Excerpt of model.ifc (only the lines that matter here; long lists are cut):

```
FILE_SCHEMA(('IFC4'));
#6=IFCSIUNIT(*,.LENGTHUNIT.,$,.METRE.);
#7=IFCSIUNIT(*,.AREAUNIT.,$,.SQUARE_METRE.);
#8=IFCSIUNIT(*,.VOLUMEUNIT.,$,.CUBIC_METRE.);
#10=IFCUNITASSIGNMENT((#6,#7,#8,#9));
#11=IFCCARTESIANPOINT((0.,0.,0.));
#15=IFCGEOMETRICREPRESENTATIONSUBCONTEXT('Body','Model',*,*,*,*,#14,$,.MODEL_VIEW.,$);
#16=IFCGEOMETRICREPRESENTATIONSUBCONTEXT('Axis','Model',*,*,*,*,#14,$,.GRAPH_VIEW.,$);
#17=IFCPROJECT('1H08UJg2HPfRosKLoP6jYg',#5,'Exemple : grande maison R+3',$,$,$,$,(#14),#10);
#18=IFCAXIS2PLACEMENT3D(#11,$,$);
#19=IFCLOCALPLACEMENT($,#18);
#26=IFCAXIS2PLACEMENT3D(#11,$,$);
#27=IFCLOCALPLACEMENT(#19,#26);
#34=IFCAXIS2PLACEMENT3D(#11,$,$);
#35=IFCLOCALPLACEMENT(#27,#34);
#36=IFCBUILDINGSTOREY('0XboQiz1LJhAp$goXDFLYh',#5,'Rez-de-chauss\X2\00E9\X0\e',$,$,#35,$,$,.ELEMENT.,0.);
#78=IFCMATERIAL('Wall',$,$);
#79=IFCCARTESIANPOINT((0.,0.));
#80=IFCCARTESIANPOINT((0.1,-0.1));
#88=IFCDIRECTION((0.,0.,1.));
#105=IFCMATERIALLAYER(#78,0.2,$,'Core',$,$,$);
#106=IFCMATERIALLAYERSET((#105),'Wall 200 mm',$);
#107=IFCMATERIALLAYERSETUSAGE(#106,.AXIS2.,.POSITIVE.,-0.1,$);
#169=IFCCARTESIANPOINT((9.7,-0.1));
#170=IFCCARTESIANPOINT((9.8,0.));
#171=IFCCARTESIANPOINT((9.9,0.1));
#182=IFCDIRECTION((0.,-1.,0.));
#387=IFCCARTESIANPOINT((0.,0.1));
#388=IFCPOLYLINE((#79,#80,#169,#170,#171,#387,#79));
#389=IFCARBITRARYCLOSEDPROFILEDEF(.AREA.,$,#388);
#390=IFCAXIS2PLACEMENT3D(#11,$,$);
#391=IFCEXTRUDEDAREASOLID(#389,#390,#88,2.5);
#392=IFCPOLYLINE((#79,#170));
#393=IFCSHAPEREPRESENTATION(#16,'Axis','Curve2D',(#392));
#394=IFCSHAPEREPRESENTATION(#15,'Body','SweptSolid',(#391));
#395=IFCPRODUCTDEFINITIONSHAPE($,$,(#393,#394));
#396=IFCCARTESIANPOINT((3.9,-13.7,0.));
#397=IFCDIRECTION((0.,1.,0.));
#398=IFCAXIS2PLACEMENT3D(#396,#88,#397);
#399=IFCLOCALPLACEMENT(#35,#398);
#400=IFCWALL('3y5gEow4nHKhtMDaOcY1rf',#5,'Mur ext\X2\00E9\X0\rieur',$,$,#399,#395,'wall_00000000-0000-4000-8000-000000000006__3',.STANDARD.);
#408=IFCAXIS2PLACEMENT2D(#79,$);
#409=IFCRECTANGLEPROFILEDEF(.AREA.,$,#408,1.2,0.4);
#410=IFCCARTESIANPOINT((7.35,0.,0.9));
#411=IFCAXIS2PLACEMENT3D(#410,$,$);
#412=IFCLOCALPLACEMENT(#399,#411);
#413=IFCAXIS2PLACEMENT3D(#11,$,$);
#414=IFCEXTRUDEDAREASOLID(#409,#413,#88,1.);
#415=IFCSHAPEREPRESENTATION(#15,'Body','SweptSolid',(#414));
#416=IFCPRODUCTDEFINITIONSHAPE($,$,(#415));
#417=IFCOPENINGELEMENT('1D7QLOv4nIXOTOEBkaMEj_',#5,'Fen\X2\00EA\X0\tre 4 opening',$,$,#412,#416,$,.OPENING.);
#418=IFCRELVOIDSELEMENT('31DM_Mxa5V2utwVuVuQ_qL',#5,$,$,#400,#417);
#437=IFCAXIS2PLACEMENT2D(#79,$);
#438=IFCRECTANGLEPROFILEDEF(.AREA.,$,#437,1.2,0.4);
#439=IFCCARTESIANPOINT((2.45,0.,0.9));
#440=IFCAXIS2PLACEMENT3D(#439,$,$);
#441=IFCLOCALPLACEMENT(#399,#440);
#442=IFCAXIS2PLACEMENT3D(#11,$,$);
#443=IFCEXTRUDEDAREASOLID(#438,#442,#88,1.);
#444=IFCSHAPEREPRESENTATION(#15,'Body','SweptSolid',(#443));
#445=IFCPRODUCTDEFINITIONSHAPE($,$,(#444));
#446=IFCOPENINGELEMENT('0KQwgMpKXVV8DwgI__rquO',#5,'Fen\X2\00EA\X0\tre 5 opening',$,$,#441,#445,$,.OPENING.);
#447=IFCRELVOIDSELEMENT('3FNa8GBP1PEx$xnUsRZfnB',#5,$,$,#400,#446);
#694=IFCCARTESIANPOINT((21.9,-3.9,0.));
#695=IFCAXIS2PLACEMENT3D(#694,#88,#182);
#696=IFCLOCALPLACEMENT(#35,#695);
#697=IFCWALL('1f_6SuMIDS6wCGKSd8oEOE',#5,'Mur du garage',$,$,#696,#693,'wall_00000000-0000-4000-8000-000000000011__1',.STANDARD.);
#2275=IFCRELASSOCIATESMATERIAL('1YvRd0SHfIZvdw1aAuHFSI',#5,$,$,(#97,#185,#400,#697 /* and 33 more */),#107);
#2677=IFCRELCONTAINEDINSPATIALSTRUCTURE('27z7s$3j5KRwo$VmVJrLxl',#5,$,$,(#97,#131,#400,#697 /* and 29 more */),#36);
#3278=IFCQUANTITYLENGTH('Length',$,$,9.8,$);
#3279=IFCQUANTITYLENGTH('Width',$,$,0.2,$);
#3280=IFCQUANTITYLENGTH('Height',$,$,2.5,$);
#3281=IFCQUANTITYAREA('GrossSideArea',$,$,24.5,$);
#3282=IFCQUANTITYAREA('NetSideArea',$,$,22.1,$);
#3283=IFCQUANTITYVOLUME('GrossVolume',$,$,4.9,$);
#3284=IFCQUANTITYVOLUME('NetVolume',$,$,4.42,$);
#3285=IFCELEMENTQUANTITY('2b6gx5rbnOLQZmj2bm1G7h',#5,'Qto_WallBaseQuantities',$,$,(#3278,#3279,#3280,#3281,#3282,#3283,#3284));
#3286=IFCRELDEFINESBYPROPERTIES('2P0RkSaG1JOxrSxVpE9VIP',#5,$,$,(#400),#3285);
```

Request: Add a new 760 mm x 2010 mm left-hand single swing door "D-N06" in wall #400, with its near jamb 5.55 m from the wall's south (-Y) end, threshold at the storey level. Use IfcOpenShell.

```python
import numpy as np
import ifcopenshell
import ifcopenshell.api.feature
import ifcopenshell.api.geometry
import ifcopenshell.api.pset
import ifcopenshell.api.root
import ifcopenshell.api.spatial
import ifcopenshell.geom
import ifcopenshell.util.element
import ifcopenshell.util.placement
import ifcopenshell.util.representation
import ifcopenshell.util.shape
import ifcopenshell.util.unit

model = ifcopenshell.open("model.ifc")
unit_scale = ifcopenshell.util.unit.calculate_unit_scale(model)
area_scale = ifcopenshell.util.unit.calculate_unit_scale(model, "AREAUNIT")
volume_scale = ifcopenshell.util.unit.calculate_unit_scale(model, "VOLUMEUNIT")
settings = ifcopenshell.geom.settings()


def volume(element):
    """Net volume in cubic metres, openings subtracted."""
    shape = ifcopenshell.geom.create_shape(settings, element)
    return ifcopenshell.util.shape.get_volume(shape.geometry)


wall = model.by_id(400)
storey = ifcopenshell.util.element.get_container(wall, ifc_class="IfcBuildingStorey")
context = ifcopenshell.util.representation.get_context(model, "Model", "Body", "MODEL_VIEW")
before = volume(wall)

width, height, from_end, sill = 0.76, 2.01, 5.55, 0.0  # metres

# The wall runs along its own X axis, and the end named is its -X end.
wall_shape = ifcopenshell.geom.create_shape(settings, wall)
x, y, z = ifcopenshell.util.shape.get_vertices(wall_shape.geometry).T
start = x.min() + from_end
face, thickness = float(y.min()), float(y.max() - y.min())
wall_matrix = ifcopenshell.util.placement.get_local_placement(wall.ObjectPlacement)
level = ifcopenshell.util.placement.get_local_placement(storey.ObjectPlacement)[2, 3]


def in_wall(x, y):
    """Placement at x, y metres in the wall's axes, at sill height."""
    matrix = wall_matrix.copy()
    matrix[:, 3] = wall_matrix @ np.array([x / unit_scale, y / unit_scale, 0.0, 1.0])
    matrix[2, 3] = level + sill / unit_scale
    return matrix


# Opening: a box that overshoots both wall faces by 50 mm.
opening = ifcopenshell.api.root.create_entity(model, ifc_class="IfcOpeningElement", predefined_type="OPENING")
box = ifcopenshell.api.geometry.add_wall_representation(
    model, context=context, length=width, height=height, thickness=thickness + 0.1
)
ifcopenshell.api.geometry.assign_representation(model, product=opening, representation=box)
ifcopenshell.api.geometry.edit_object_placement(model, product=opening, matrix=in_wall(start, face - 0.05), is_si=False)
ifcopenshell.api.feature.add_feature(model, feature=opening, element=wall)

door = ifcopenshell.api.root.create_entity(model, ifc_class="IfcDoor", name="D-N06", predefined_type="DOOR")
door.OverallWidth, door.OverallHeight = width / unit_scale, height / unit_scale
door.OperationType = "SINGLE_SWING_LEFT"
body = ifcopenshell.api.geometry.add_door_representation(
    model,
    context=context,
    overall_width=door.OverallWidth,
    overall_height=door.OverallHeight,
    operation_type="SINGLE_SWING_LEFT",
    lining_properties={"LiningDepth": thickness / unit_scale, "ThresholdDepth": thickness / unit_scale},
)
ifcopenshell.api.geometry.assign_representation(model, product=door, representation=body)
ifcopenshell.api.spatial.assign_container(model, products=[door], relating_structure=storey)
ifcopenshell.api.feature.add_filling(model, opening=opening, element=door)

# The lining spans the wall, so the door starts at the wall face.
ifcopenshell.api.geometry.edit_object_placement(model, product=door, matrix=in_wall(start, face), is_si=False)

after = volume(wall)

# Update the wall's stored quantities.
qto = model.by_id(ifcopenshell.util.element.get_pset(wall, "Qto_WallBaseQuantities", should_inherit=False)["id"])
ifcopenshell.api.pset.edit_qto(model, qto=qto, properties={
    "NetSideArea": after / thickness / area_scale,
    "NetVolume": after / volume_scale,
})

print(f"wall volume {before:.3f} -> {after:.3f} m3")

model.write("model-out.ifc")
```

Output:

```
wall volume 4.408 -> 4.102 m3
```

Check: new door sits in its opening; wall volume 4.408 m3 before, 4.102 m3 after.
